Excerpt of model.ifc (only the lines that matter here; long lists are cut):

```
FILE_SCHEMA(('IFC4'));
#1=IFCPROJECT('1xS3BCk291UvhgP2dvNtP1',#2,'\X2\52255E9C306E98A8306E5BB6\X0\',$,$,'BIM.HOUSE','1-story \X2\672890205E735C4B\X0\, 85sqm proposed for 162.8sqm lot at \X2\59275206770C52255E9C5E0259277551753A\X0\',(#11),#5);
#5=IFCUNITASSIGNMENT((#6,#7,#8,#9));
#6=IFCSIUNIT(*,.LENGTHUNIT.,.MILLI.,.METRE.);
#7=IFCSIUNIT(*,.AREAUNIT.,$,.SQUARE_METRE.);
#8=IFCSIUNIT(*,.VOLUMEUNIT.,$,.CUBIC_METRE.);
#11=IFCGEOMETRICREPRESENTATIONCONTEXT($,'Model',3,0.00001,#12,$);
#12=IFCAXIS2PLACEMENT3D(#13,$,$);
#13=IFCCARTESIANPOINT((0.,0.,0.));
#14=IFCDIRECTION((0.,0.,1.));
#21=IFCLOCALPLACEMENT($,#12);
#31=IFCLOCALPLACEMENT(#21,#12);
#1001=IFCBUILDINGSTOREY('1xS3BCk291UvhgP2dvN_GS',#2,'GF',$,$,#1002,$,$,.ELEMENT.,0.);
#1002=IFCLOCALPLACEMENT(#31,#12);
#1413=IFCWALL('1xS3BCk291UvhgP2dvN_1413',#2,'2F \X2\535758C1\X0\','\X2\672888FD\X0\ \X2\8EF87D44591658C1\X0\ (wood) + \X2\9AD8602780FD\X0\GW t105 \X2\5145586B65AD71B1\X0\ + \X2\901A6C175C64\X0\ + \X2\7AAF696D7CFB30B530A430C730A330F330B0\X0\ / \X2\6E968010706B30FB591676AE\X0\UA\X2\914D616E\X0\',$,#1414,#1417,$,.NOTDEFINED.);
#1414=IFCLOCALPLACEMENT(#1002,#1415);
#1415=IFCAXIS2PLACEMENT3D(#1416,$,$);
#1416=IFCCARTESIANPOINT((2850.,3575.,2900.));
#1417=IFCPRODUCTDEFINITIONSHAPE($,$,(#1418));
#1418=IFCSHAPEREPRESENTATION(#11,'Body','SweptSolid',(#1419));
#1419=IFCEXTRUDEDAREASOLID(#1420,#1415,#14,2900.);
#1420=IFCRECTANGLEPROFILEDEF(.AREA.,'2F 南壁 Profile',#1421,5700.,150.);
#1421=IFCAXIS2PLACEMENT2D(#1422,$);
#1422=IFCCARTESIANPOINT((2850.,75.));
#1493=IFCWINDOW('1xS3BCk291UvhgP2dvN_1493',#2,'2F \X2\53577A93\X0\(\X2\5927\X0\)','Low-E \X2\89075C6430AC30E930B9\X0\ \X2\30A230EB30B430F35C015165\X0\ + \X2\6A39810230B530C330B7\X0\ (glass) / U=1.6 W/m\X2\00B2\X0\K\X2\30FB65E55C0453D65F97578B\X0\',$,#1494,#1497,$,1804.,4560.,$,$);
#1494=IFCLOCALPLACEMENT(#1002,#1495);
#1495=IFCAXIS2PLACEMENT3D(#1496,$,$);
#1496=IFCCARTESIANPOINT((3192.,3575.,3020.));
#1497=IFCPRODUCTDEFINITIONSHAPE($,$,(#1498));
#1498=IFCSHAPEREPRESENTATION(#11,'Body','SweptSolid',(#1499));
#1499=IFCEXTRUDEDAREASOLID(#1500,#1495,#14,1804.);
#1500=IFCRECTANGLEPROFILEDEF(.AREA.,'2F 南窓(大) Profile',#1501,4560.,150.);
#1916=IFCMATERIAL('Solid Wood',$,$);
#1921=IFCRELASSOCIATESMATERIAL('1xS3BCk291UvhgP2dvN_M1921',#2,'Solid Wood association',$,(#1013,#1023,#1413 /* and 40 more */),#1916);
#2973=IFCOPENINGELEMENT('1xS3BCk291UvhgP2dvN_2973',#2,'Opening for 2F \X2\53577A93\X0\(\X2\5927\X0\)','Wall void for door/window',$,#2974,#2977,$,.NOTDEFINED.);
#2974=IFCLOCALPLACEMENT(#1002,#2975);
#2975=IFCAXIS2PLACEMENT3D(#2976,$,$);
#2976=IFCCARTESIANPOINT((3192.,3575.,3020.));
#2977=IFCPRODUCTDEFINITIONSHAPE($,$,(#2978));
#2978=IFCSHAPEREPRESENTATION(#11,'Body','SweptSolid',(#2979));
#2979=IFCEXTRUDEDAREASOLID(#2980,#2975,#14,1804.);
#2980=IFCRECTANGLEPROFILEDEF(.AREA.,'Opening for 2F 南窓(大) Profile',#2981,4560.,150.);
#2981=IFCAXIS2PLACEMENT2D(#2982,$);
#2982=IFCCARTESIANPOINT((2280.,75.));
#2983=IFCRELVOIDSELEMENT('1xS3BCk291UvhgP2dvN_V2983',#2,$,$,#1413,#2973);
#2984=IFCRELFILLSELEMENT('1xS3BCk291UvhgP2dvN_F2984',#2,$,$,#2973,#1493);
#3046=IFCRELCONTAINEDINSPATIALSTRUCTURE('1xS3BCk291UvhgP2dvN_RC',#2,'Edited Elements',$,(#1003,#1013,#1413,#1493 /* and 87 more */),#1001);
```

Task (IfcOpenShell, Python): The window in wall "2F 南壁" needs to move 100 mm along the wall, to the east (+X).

```python
import ifcopenshell
import ifcopenshell.api.geometry
import ifcopenshell.util.placement

model = ifcopenshell.open("model.ifc")

window = model.by_id(1493)
opening = window.FillsVoids[0].RelatingOpeningElement
wall = opening.VoidsElements[0].RelatingBuildingElement

wall_matrix = ifcopenshell.util.placement.get_local_placement(wall.ObjectPlacement)
shift = wall_matrix[:3, 0] * 100.0
before = ifcopenshell.util.placement.get_local_placement(window.ObjectPlacement)[:3, 3].copy()

# The window is not placed relative to its opening, so move both.
for product in (opening, window):
    matrix = ifcopenshell.util.placement.get_local_placement(product.ObjectPlacement)
    matrix[:3, 3] += shift
    ifcopenshell.api.geometry.edit_object_placement(model, product=product, matrix=matrix, is_si=False)

after = ifcopenshell.util.placement.get_local_placement(window.ObjectPlacement)[:3, 3]
print("window moved by", (after - before).round(3) + 0.0)

model.write("model_updated.ifc")
```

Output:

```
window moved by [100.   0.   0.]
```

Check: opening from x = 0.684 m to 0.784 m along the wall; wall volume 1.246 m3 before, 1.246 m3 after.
